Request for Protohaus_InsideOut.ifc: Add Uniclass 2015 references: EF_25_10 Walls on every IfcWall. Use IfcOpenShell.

First a look at what the model holds.

```python
import ifcopenshell

model = ifcopenshell.open("Protohaus_InsideOut.ifc")
print(model.schema)
print("classifications:", [c.Name for c in model.by_type("IfcClassification")])
for ifc_class in ("IfcDoor", "IfcRoof", "IfcStair", "IfcWall", "IfcWindow"):
    print(ifc_class, len(model.by_type(ifc_class)))
```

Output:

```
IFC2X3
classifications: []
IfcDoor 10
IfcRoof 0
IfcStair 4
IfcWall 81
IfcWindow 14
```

```python
import ifcopenshell
import ifcopenshell.api.classification

model = ifcopenshell.open("Protohaus_InsideOut.ifc")

# IFC2X3 requires Source and Edition and has no link from the project to the system.
system = model.create_entity("IfcClassification", Source="NBS", Edition="2015", Name="Uniclass 2015")

codes = {
    "IfcWall": ("EF_25_10", "Walls"),
}
for ifc_class, (code, name) in codes.items():
    products = model.by_type(ifc_class)
    ifcopenshell.api.classification.add_reference(
        model, products=products, classification=system, identification=code, name=name
    )
    print(code, len(products))

model.write("Protohaus_InsideOut_updated.ifc")
```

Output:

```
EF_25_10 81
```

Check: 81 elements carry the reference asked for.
